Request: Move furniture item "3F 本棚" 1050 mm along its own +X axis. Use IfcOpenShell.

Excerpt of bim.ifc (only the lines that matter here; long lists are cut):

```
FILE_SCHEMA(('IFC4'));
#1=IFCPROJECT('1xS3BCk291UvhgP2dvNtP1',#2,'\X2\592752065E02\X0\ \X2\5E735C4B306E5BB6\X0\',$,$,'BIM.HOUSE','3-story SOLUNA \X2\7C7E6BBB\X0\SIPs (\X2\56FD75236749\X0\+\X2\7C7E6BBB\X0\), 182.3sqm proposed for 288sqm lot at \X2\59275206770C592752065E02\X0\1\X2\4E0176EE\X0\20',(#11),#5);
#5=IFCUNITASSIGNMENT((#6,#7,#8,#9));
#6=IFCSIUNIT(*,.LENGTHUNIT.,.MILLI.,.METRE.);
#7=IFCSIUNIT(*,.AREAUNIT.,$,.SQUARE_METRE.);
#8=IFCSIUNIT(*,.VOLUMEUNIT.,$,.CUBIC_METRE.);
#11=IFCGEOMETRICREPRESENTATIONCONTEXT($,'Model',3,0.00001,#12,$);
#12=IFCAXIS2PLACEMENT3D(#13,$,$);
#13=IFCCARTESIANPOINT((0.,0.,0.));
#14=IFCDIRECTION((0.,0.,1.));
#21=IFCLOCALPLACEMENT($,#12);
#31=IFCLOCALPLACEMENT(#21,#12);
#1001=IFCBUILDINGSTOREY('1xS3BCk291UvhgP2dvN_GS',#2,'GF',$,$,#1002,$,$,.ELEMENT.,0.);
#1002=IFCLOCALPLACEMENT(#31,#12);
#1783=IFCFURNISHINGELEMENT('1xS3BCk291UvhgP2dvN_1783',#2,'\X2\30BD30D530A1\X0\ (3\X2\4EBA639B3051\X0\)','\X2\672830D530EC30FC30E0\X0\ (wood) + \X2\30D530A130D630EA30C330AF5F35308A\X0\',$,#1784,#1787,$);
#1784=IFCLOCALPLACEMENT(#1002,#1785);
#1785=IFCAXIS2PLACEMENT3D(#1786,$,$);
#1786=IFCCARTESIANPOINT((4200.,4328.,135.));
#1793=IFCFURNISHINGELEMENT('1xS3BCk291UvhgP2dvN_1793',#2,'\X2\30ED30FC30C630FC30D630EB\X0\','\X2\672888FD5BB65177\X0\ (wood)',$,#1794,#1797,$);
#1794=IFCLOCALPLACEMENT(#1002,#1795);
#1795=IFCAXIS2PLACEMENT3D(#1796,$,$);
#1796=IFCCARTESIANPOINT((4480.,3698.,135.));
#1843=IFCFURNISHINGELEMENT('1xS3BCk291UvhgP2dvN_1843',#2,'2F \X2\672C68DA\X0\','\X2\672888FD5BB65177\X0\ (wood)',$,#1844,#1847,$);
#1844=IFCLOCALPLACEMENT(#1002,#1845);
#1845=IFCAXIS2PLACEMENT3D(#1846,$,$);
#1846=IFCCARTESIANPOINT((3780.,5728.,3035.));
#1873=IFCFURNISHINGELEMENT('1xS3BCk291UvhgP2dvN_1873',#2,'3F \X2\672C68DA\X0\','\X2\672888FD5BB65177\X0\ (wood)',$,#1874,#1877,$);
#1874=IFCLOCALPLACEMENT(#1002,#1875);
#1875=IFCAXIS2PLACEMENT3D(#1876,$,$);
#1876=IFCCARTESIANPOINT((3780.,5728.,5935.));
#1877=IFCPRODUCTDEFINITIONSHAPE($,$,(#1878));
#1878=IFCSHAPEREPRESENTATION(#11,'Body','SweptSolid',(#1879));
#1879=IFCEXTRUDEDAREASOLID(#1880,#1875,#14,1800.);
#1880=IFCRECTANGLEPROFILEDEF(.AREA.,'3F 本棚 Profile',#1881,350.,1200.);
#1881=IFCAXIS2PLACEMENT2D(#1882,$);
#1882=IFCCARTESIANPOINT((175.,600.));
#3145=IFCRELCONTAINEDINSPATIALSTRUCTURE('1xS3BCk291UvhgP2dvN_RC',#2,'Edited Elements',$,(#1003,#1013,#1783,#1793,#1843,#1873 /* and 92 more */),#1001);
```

```python
import ifcopenshell
import ifcopenshell.api.geometry
import ifcopenshell.util.placement

model = ifcopenshell.open("bim.ifc")

item = model.by_id(1873)
matrix = ifcopenshell.util.placement.get_local_placement(item.ObjectPlacement)
matrix[:3, 3] += matrix[:3, 0] * 1050.0
ifcopenshell.api.geometry.edit_object_placement(model, product=item, matrix=matrix, is_si=False)

print(ifcopenshell.util.placement.get_local_placement(item.ObjectPlacement).round(3) + 0.0)

model.write("bim_updated.ifc")
```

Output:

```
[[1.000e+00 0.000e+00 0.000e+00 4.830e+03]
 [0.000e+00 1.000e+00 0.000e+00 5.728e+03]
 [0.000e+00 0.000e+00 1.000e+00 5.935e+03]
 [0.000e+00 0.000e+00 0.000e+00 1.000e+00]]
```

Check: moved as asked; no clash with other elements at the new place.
